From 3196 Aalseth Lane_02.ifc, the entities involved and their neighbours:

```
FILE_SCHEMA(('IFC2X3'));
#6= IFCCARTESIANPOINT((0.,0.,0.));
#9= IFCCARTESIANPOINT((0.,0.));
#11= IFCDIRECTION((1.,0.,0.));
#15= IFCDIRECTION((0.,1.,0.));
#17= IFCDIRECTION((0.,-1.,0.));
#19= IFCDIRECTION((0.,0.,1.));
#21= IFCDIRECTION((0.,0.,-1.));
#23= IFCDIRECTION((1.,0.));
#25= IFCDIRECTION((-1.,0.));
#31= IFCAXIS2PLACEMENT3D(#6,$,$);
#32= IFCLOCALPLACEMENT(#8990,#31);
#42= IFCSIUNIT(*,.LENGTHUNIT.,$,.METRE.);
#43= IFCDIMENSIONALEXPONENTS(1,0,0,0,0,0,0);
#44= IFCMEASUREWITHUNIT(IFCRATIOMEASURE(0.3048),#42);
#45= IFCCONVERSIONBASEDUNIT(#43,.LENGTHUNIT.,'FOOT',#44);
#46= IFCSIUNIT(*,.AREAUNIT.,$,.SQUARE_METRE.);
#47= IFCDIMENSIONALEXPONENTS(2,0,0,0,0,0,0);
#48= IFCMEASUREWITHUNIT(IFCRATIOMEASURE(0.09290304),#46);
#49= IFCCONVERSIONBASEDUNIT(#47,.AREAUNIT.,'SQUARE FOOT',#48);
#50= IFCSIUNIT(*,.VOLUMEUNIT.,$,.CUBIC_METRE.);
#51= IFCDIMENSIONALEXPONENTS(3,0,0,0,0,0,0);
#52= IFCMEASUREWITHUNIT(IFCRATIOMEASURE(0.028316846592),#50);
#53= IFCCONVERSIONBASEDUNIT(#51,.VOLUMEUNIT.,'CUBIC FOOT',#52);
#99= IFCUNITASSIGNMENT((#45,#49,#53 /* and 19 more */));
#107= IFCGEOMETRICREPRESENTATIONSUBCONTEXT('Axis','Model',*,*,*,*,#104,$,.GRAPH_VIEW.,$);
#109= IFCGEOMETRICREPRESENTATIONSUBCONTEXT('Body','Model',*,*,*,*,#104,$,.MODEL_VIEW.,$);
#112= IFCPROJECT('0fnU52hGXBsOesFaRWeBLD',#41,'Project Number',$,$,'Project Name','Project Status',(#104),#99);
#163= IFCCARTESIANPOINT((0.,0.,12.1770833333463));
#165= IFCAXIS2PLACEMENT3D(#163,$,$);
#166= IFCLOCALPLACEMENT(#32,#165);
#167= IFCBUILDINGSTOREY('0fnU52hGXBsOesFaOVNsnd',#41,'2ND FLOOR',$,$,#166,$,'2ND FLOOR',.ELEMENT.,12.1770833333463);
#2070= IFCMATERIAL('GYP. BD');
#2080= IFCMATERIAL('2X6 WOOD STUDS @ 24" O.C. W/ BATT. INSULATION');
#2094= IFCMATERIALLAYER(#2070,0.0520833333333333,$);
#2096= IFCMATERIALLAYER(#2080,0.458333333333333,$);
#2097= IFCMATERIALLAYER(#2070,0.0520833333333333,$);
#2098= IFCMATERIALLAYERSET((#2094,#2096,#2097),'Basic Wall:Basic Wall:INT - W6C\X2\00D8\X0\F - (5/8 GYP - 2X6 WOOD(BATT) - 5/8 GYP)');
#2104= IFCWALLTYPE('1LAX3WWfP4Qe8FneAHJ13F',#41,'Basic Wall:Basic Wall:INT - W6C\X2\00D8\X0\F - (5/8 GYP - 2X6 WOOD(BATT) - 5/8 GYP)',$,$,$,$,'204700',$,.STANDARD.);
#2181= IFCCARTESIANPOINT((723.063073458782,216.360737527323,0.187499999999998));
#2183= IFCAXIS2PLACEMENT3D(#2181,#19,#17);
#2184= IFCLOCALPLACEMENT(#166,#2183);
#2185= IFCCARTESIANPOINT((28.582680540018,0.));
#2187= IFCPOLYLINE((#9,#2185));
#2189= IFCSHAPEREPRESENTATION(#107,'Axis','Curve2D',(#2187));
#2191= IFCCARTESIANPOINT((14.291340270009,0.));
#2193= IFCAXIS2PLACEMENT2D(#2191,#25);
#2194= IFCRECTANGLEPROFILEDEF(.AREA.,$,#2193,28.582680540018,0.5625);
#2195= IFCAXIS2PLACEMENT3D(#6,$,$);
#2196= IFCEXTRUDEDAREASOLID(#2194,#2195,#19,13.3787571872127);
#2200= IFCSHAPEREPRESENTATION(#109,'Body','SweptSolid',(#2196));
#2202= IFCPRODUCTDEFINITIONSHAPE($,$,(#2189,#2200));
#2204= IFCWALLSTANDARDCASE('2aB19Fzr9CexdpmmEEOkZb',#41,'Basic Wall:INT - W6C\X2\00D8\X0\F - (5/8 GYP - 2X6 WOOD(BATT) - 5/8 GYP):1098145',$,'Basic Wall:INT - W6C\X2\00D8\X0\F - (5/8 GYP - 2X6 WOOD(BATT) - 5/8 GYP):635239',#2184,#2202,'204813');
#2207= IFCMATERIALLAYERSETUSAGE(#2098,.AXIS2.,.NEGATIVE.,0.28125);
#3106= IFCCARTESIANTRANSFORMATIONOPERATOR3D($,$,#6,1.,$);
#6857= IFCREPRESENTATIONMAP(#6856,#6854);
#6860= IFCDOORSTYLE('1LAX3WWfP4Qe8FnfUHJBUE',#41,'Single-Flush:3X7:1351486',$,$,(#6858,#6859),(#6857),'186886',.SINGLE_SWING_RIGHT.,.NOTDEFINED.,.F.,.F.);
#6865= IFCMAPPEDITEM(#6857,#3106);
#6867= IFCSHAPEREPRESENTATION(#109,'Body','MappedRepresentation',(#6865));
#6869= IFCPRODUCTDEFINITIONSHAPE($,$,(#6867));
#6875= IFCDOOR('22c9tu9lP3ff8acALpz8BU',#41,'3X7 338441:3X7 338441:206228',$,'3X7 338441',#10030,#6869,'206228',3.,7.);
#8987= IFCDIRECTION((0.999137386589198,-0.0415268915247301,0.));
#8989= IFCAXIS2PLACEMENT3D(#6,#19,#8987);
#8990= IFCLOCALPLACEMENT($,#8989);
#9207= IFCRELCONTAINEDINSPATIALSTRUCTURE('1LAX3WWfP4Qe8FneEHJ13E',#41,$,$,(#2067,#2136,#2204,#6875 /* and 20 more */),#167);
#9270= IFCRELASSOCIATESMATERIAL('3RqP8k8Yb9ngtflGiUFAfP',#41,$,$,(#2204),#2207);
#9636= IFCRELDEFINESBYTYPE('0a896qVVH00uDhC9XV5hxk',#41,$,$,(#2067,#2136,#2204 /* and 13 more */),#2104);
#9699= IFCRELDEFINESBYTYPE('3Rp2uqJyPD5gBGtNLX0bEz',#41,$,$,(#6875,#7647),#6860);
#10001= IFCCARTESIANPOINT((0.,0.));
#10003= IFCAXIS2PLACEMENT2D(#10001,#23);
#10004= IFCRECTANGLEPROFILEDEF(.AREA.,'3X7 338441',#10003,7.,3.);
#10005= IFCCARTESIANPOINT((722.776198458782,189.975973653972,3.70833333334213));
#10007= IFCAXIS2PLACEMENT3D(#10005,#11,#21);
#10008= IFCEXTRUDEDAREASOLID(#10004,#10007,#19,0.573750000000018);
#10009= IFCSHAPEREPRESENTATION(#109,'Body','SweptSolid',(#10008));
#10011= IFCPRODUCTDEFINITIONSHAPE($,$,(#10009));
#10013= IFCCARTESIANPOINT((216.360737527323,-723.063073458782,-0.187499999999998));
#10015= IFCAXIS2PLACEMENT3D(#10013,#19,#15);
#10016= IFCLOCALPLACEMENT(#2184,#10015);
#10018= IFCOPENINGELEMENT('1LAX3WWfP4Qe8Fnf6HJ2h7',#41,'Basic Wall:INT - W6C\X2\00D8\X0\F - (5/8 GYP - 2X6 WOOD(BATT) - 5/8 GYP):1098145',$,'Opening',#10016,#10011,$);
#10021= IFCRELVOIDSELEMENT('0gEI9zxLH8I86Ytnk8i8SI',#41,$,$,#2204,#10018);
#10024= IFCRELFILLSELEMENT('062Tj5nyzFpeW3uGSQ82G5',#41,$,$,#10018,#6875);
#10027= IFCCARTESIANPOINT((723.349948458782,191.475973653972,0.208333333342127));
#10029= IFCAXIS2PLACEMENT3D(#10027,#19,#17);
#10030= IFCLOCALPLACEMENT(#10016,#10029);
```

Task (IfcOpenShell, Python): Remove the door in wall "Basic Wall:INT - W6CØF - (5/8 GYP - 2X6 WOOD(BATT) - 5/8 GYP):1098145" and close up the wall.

```python
import ifcopenshell
import ifcopenshell.api.feature
import ifcopenshell.api.root
import ifcopenshell.geom
import ifcopenshell.util.shape

model = ifcopenshell.open("3196 Aalseth Lane_02.ifc")
settings = ifcopenshell.geom.settings()


def volume(element):
    """Net volume in cubic metres, openings subtracted."""
    shape = ifcopenshell.geom.create_shape(settings, element)
    return ifcopenshell.util.shape.get_volume(shape.geometry)


door = model.by_id(6875)
opening = door.FillsVoids[0].RelatingOpeningElement
wall = opening.VoidsElements[0].RelatingBuildingElement
before = volume(wall)

ifcopenshell.api.root.remove_product(model, product=door)
ifcopenshell.api.feature.remove_feature(model, feature=opening)

after = volume(wall)

print(f"wall volume {before:.3f} -> {after:.3f} m3")

model.write("3196 Aalseth Lane_02_v2.ifc")
```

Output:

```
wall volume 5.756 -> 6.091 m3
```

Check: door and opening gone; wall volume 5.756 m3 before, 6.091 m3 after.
